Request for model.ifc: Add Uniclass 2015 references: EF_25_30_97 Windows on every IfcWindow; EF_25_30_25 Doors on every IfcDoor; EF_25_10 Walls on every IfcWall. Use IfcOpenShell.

First a look at what the model holds.

```python
import ifcopenshell

model = ifcopenshell.open("model.ifc")
print(model.schema)
print("classifications:", [c.Name for c in model.by_type("IfcClassification")])
for ifc_class in ("IfcDoor", "IfcRoof", "IfcStair", "IfcWall", "IfcWindow"):
    print(ifc_class, len(model.by_type(ifc_class)))
```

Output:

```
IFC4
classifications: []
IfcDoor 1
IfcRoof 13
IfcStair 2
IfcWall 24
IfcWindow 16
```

```python
import ifcopenshell
import ifcopenshell.api.classification

model = ifcopenshell.open("model.ifc")

system = ifcopenshell.api.classification.add_classification(model, classification="Uniclass 2015")

codes = {
    "IfcWindow": ("EF_25_30_97", "Windows"),
    "IfcDoor": ("EF_25_30_25", "Doors"),
    "IfcWall": ("EF_25_10", "Walls"),
}
for ifc_class, (code, name) in codes.items():
    products = model.by_type(ifc_class)
    ifcopenshell.api.classification.add_reference(
        model, products=products, classification=system, identification=code, name=name
    )
    print(code, len(products))

model.write("model_updated.ifc")
```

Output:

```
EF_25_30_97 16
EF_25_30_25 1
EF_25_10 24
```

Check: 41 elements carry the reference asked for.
